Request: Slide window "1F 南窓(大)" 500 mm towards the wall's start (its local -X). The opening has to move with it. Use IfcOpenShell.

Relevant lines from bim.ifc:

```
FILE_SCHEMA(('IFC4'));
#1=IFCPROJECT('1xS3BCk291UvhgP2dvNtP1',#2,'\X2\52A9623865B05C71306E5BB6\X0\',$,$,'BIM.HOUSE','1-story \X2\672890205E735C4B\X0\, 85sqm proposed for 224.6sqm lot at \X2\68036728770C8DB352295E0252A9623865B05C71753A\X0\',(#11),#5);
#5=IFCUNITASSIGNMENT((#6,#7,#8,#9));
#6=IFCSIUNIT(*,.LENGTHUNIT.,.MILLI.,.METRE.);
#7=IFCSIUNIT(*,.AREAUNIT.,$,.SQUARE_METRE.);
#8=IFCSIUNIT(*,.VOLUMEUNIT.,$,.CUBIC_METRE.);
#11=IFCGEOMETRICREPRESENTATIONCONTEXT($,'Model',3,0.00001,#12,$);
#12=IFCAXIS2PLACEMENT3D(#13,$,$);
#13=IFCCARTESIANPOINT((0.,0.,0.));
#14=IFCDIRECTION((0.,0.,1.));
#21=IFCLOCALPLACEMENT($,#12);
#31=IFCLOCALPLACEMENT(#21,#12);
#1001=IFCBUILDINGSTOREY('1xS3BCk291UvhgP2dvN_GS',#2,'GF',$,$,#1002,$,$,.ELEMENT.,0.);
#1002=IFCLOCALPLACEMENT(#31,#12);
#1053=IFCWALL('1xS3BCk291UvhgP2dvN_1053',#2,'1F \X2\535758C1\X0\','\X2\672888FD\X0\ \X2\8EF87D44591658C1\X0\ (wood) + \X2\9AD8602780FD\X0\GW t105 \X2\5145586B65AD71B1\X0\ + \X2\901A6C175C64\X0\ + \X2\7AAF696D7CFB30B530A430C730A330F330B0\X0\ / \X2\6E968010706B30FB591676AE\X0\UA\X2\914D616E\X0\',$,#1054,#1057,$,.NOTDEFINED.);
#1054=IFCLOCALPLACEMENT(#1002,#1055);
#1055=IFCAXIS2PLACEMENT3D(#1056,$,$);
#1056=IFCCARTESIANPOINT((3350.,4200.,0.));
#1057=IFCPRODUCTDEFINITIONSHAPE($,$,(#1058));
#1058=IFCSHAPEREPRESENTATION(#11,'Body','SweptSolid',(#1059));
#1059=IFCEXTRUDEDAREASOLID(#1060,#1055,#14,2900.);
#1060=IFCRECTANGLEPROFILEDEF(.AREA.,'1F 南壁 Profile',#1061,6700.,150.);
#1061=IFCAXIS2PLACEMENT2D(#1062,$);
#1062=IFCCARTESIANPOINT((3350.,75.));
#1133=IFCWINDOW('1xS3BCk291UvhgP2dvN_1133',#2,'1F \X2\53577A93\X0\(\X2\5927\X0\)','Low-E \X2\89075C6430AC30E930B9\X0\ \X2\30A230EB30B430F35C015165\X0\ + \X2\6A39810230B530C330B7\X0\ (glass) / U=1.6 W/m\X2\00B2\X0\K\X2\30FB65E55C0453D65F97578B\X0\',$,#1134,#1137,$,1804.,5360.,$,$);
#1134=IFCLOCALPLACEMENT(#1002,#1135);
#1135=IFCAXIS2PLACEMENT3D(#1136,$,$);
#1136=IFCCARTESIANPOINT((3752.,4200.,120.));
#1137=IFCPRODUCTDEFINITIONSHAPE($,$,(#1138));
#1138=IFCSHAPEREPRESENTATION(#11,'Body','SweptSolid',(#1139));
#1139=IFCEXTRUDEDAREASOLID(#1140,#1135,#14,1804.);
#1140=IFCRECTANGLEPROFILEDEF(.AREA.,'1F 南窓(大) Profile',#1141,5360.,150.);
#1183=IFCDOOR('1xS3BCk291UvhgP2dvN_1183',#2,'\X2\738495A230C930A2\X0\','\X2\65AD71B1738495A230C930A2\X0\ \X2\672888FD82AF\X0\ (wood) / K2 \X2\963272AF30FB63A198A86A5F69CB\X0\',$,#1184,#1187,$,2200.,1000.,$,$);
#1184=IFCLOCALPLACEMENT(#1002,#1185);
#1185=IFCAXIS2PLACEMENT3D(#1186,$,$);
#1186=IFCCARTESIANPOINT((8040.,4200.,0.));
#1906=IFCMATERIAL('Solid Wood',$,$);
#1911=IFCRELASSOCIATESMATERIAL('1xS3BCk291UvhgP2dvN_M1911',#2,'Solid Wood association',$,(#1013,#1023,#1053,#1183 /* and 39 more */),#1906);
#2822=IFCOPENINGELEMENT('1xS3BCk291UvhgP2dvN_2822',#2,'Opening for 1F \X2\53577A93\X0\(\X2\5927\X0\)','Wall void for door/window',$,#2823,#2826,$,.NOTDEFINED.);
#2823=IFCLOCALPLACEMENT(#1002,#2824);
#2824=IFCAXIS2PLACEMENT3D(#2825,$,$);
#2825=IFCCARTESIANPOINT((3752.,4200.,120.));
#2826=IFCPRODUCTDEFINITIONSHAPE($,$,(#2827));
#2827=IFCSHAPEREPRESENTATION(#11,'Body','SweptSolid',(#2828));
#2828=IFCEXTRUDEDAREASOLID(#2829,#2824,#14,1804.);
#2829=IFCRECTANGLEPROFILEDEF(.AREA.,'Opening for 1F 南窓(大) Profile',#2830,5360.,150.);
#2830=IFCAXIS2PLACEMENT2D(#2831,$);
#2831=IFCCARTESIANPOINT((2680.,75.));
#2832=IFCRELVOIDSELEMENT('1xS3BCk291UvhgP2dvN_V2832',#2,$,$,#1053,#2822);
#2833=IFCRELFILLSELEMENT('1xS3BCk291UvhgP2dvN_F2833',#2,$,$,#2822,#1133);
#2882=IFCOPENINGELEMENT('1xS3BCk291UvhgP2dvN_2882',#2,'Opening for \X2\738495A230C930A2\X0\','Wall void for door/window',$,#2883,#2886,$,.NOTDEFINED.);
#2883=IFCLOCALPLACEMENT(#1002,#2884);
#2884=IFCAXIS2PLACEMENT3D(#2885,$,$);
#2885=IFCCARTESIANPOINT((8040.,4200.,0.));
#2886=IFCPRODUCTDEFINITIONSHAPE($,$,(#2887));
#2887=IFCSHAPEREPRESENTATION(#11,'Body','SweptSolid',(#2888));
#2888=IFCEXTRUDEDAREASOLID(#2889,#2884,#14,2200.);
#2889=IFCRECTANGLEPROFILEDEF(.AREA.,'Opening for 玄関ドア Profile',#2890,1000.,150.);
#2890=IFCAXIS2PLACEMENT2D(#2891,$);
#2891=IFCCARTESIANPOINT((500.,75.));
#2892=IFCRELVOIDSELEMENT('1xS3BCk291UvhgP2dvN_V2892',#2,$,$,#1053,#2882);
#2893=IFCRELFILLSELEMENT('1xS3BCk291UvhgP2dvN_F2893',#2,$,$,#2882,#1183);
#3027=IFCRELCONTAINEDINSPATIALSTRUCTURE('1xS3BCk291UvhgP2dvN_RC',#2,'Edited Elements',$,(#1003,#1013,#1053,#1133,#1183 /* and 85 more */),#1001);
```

```python
import ifcopenshell
import ifcopenshell.api.geometry
import ifcopenshell.util.placement
import ifcopenshell.util.unit

model = ifcopenshell.open("bim.ifc")
unit_scale = ifcopenshell.util.unit.calculate_unit_scale(model)

window = model.by_guid("1xS3BCk291UvhgP2dvN_1133")
opening = window.FillsVoids[0].RelatingOpeningElement
wall = opening.VoidsElements[0].RelatingBuildingElement

wall_matrix = ifcopenshell.util.placement.get_local_placement(wall.ObjectPlacement)
shift = wall_matrix[:3, 0] * -0.5 / unit_scale
before = ifcopenshell.util.placement.get_local_placement(window.ObjectPlacement)[:3, 3].copy()

# The window is not placed relative to its opening, so move both.
for product in (opening, window):
    matrix = ifcopenshell.util.placement.get_local_placement(product.ObjectPlacement)
    matrix[:3, 3] += shift
    ifcopenshell.api.geometry.edit_object_placement(model, product=product, matrix=matrix, is_si=False)

after = ifcopenshell.util.placement.get_local_placement(window.ObjectPlacement)[:3, 3]
print("window moved by", (after - before).round(3) + 0.0)

model.write("bim_edited.ifc")
```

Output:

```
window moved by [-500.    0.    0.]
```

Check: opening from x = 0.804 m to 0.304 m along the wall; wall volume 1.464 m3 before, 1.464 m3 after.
